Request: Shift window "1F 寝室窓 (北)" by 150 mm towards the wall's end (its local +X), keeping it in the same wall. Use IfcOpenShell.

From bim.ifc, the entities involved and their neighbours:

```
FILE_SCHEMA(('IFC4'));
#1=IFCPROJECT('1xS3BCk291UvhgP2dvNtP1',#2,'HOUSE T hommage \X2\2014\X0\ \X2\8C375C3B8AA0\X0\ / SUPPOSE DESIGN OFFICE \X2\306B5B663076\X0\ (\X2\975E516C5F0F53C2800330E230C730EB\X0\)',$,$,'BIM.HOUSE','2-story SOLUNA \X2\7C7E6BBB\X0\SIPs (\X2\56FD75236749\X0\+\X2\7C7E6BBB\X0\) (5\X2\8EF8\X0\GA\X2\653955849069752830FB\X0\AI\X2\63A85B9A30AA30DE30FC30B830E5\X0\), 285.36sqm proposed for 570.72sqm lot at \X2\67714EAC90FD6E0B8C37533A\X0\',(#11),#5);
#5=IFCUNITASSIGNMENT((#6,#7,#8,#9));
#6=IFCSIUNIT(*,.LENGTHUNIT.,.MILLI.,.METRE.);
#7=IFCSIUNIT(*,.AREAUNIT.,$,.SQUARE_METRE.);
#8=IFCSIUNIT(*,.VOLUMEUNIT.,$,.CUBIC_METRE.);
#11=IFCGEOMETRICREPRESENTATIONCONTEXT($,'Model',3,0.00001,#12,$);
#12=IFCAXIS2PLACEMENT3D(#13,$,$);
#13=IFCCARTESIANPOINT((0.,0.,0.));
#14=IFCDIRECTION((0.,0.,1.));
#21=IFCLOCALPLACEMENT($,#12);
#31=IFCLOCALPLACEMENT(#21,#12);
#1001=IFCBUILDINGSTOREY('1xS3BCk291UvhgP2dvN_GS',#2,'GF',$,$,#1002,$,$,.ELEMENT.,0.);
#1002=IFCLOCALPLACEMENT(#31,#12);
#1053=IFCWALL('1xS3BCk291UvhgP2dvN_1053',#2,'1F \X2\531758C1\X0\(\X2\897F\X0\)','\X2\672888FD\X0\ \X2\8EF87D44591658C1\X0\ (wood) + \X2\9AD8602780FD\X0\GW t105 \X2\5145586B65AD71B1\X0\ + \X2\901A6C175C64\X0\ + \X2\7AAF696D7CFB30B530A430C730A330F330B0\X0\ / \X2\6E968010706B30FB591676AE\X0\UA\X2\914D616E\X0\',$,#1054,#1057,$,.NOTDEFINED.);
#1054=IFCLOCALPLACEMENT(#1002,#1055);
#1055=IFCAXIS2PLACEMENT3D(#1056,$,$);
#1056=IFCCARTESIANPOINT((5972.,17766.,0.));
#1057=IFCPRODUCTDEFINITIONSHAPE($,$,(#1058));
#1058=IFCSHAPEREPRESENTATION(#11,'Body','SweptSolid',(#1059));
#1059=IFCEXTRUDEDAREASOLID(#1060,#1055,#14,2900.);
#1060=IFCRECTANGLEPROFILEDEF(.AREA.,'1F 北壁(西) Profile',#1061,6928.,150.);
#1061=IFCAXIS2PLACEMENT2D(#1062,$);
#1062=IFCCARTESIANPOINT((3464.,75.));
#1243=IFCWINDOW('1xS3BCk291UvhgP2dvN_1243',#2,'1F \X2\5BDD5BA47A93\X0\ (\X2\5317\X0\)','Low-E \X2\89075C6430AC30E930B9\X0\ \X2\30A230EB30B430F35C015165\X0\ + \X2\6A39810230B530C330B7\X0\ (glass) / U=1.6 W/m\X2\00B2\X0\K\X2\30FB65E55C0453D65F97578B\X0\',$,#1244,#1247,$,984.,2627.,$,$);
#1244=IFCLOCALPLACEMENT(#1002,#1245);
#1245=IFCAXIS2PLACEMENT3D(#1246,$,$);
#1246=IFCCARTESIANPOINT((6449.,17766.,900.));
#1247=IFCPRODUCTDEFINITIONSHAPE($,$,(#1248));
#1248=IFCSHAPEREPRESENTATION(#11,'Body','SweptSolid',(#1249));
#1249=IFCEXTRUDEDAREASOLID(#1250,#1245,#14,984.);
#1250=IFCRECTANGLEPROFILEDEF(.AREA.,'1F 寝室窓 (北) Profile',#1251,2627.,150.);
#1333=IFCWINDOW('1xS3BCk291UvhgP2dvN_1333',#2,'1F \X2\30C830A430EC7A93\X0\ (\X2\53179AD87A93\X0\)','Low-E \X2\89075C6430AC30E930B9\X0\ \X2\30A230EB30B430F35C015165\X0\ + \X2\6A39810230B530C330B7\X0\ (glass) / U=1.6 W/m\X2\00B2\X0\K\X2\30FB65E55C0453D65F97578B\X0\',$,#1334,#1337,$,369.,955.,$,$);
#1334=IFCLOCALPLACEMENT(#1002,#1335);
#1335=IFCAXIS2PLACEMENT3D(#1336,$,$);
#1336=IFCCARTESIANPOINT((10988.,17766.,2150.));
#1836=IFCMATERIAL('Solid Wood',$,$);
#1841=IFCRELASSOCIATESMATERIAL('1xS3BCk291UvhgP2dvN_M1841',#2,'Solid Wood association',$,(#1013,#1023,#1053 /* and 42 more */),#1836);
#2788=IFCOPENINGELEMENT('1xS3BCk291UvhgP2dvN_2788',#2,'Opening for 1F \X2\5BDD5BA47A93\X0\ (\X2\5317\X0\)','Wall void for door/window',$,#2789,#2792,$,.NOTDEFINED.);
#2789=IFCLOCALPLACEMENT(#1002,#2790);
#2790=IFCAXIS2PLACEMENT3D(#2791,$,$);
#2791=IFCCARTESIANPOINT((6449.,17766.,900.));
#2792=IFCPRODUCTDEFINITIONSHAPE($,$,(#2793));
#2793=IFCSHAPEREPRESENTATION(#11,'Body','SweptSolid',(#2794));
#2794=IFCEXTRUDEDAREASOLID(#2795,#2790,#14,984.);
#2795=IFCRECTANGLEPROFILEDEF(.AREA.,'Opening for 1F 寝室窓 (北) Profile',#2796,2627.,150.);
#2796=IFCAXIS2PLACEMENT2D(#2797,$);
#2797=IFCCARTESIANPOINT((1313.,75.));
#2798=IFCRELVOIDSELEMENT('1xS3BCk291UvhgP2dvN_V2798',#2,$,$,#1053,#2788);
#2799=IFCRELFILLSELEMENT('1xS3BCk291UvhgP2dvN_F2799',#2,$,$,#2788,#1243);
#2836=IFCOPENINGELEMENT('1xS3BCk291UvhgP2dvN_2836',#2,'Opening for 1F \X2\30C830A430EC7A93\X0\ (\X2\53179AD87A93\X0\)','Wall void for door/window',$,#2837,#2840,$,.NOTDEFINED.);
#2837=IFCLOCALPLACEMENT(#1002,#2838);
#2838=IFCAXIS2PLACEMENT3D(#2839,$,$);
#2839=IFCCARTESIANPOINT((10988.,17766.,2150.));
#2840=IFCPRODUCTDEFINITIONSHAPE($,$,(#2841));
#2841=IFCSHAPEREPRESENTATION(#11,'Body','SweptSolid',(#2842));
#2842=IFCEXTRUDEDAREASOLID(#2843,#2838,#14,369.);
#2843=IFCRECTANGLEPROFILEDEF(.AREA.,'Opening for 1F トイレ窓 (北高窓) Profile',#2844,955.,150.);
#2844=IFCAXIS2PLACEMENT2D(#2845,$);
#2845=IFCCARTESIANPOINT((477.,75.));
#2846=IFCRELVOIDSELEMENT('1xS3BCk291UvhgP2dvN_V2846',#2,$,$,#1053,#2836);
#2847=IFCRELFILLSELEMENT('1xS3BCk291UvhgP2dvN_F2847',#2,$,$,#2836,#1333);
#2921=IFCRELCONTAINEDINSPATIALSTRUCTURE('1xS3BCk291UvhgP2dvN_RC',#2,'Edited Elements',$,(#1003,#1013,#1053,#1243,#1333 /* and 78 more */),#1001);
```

```python
import ifcopenshell
import ifcopenshell.api.geometry
import ifcopenshell.util.placement

model = ifcopenshell.open("bim.ifc")

window = model.by_guid("1xS3BCk291UvhgP2dvN_1243")
opening = window.FillsVoids[0].RelatingOpeningElement
wall = opening.VoidsElements[0].RelatingBuildingElement

wall_matrix = ifcopenshell.util.placement.get_local_placement(wall.ObjectPlacement)
shift = wall_matrix[:3, 0] * 150.0
before = ifcopenshell.util.placement.get_local_placement(window.ObjectPlacement)[:3, 3].copy()

# The window is not placed relative to its opening, so move both.
for product in (opening, window):
    matrix = ifcopenshell.util.placement.get_local_placement(product.ObjectPlacement)
    matrix[:3, 3] += shift
    ifcopenshell.api.geometry.edit_object_placement(model, product=product, matrix=matrix, is_si=False)

after = ifcopenshell.util.placement.get_local_placement(window.ObjectPlacement)[:3, 3]
print("window moved by", (after - before).round(3) + 0.0)

model.write("bim_updated.ifc")
```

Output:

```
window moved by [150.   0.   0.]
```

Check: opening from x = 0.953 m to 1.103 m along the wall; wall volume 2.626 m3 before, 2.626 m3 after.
